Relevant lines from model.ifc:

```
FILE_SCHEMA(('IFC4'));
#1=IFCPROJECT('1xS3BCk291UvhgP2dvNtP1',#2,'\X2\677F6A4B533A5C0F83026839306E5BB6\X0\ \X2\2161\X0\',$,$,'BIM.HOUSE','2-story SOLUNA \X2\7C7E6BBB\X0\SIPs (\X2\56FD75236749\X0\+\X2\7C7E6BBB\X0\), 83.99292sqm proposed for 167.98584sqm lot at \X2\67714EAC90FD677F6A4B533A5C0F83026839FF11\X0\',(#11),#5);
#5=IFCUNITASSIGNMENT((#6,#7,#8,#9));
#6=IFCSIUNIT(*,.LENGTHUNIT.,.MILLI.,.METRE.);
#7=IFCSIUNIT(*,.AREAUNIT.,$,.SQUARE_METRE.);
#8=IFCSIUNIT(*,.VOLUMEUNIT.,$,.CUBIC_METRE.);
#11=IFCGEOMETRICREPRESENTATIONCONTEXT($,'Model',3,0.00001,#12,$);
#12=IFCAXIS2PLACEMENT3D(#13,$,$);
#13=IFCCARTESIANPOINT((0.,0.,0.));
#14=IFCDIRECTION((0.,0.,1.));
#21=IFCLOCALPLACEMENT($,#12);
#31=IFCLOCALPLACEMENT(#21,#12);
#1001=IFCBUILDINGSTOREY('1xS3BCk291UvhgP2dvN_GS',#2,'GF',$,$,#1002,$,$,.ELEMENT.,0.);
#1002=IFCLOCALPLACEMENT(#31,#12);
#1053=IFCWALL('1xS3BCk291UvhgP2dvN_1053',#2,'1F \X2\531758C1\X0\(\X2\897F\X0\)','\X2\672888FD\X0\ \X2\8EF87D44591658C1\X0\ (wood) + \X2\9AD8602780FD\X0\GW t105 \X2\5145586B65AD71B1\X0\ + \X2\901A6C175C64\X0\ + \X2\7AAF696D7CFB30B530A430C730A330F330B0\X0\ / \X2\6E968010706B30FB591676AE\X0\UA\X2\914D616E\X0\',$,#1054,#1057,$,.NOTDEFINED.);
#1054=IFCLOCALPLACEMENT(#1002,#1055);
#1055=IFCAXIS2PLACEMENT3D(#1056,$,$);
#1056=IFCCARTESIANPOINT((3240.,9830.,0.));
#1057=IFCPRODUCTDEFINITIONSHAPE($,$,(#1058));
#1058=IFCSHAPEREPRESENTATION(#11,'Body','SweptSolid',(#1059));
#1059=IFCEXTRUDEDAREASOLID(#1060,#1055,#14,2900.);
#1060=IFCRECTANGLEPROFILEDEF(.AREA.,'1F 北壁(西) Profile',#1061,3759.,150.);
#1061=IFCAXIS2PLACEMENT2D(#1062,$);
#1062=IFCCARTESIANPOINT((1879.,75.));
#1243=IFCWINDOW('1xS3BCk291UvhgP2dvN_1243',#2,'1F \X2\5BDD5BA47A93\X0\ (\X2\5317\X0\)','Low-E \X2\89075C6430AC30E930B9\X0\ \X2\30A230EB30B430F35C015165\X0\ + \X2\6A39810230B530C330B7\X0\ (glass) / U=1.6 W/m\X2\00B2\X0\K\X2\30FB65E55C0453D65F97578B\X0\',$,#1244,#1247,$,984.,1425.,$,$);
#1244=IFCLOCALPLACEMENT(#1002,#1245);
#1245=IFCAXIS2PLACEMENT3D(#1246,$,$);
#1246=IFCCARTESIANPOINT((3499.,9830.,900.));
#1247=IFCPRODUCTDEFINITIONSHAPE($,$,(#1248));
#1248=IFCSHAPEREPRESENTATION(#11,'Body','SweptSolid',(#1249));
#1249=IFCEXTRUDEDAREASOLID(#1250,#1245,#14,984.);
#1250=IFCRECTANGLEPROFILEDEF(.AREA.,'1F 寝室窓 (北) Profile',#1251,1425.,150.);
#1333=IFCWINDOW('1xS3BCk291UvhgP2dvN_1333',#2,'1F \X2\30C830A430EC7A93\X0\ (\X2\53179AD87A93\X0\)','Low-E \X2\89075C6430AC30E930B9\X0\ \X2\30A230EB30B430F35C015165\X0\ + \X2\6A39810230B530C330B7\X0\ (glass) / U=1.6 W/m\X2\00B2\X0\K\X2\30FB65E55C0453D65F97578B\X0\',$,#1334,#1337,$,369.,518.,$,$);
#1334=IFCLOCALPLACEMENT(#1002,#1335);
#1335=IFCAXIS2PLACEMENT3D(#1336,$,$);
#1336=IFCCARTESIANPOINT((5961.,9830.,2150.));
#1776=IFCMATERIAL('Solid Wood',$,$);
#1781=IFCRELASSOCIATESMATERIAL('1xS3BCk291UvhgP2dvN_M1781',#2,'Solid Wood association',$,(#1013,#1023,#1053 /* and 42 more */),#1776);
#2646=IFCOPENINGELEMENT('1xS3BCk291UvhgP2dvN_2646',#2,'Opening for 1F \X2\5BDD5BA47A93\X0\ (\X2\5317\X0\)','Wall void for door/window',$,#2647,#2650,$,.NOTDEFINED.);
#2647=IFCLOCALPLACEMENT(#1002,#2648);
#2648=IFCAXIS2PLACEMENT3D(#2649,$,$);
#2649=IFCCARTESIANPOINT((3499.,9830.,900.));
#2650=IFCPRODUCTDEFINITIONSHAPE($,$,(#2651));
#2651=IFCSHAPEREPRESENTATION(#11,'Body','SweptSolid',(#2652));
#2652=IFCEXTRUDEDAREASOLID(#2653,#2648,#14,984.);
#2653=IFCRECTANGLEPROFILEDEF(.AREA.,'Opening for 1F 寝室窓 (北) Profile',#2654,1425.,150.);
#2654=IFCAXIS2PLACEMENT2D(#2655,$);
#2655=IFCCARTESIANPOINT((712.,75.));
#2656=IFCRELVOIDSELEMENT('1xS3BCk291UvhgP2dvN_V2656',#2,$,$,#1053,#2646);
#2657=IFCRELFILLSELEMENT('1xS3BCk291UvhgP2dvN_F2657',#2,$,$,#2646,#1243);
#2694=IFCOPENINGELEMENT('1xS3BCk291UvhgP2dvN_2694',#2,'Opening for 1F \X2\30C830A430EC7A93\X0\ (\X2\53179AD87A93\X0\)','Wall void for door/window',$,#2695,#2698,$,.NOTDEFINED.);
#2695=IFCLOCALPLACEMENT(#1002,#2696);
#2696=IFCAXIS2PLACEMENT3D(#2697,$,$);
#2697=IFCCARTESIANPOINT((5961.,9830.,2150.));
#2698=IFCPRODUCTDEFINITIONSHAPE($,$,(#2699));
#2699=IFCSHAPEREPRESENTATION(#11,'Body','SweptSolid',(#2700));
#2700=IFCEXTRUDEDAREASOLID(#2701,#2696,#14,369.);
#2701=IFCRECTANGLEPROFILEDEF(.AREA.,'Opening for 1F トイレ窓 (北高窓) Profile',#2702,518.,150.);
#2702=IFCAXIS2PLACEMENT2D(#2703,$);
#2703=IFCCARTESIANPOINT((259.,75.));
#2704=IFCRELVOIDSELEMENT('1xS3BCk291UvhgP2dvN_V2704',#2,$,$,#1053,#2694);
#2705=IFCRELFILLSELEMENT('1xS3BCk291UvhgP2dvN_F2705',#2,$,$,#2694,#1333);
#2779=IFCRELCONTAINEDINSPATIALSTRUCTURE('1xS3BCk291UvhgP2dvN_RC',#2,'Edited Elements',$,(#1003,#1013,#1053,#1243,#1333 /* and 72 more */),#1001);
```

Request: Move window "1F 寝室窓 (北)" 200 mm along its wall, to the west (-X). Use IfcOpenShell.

```python
import ifcopenshell
import ifcopenshell.api.geometry
import ifcopenshell.util.placement

model = ifcopenshell.open("model.ifc")

window = model.by_guid("1xS3BCk291UvhgP2dvN_1243")
opening = window.FillsVoids[0].RelatingOpeningElement
wall = opening.VoidsElements[0].RelatingBuildingElement

wall_matrix = ifcopenshell.util.placement.get_local_placement(wall.ObjectPlacement)
shift = wall_matrix[:3, 0] * -200.0
before = ifcopenshell.util.placement.get_local_placement(window.ObjectPlacement)[:3, 3].copy()

# The window is not placed relative to its opening, so move both.
for product in (opening, window):
    matrix = ifcopenshell.util.placement.get_local_placement(product.ObjectPlacement)
    matrix[:3, 3] += shift
    ifcopenshell.api.geometry.edit_object_placement(model, product=product, matrix=matrix, is_si=False)

after = ifcopenshell.util.placement.get_local_placement(window.ObjectPlacement)[:3, 3]
print("window moved by", (after - before).round(3) + 0.0)

model.write("model_v2.ifc")
```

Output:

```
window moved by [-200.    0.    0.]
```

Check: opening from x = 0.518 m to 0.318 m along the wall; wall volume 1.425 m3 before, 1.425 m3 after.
